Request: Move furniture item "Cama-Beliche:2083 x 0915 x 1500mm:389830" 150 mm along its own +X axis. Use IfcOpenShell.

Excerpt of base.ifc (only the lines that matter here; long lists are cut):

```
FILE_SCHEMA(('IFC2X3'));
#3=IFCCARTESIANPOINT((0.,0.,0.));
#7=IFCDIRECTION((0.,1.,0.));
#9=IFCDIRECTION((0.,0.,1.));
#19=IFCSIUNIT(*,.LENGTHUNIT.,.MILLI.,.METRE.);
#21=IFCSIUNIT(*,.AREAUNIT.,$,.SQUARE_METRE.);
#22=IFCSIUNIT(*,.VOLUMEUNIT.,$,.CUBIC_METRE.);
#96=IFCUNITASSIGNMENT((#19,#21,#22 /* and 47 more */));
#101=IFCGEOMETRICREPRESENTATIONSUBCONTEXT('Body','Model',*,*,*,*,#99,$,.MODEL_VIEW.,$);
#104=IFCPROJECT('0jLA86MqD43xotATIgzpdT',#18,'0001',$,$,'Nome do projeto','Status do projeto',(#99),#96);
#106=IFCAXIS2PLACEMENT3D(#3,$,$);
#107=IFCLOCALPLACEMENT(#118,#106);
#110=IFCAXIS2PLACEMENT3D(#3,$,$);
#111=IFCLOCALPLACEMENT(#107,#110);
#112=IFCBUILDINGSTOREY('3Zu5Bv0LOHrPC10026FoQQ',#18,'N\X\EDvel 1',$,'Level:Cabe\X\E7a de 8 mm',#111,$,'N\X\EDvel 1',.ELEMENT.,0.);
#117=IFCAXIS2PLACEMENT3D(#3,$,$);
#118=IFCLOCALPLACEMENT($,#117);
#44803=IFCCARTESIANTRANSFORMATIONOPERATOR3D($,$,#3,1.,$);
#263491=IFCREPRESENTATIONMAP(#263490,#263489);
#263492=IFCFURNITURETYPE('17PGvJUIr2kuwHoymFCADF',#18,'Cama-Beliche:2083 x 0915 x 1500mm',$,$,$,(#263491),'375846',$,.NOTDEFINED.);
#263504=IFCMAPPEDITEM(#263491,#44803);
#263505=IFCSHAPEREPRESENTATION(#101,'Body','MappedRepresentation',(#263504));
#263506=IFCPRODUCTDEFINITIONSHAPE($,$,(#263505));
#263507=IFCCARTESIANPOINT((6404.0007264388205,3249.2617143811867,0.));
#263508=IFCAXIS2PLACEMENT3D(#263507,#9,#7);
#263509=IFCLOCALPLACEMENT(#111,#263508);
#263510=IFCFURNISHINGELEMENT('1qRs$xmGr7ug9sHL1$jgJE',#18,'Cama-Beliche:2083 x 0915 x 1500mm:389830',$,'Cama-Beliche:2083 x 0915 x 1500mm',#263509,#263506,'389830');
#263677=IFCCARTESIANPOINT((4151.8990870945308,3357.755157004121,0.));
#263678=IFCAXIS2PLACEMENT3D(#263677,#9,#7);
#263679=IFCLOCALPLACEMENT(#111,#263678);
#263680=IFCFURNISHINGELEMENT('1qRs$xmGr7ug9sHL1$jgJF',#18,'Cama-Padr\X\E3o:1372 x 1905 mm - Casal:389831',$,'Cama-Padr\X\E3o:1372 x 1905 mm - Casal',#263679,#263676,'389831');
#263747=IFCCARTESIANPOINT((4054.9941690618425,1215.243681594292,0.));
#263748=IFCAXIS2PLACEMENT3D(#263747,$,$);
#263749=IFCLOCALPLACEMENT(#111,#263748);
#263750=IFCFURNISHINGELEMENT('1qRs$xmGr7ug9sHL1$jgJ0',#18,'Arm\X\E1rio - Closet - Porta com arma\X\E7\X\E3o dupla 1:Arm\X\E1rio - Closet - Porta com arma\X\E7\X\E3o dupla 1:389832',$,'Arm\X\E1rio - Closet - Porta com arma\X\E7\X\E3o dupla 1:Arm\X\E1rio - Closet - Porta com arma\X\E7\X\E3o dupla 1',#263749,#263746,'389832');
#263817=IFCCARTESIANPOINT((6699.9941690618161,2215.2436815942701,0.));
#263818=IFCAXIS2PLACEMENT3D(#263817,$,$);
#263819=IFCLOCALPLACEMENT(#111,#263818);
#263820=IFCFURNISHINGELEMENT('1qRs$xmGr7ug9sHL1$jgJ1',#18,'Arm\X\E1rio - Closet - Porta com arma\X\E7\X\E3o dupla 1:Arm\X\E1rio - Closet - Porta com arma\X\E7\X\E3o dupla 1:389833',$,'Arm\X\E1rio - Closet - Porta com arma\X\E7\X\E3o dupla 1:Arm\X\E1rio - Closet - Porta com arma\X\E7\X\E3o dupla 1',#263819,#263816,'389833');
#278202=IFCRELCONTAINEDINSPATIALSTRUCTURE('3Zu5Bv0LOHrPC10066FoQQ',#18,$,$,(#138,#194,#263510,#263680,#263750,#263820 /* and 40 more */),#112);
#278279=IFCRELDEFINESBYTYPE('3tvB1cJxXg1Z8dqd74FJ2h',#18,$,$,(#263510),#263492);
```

```python
import ifcopenshell
import ifcopenshell.api.geometry
import ifcopenshell.util.placement
import ifcopenshell.util.unit

model = ifcopenshell.open("base.ifc")
unit_scale = ifcopenshell.util.unit.calculate_unit_scale(model)

item = model.by_id(263510)
matrix = ifcopenshell.util.placement.get_local_placement(item.ObjectPlacement)
matrix[:3, 3] += matrix[:3, 0] * 0.15 / unit_scale
ifcopenshell.api.geometry.edit_object_placement(model, product=item, matrix=matrix, is_si=False)

print(ifcopenshell.util.placement.get_local_placement(item.ObjectPlacement).round(3) + 0.0)

model.write("base-out.ifc")
```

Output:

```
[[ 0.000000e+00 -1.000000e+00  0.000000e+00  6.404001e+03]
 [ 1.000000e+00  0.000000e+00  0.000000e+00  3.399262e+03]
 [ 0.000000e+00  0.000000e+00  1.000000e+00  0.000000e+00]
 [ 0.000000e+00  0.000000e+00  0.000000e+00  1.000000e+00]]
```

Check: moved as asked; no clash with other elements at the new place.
